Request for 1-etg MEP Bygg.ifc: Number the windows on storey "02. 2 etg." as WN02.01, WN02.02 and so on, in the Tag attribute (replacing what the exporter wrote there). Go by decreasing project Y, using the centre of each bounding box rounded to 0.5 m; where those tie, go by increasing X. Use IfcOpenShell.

First a look at what the model holds.

```python
import ifcopenshell
import ifcopenshell.util.element
import ifcopenshell.util.placement

model = ifcopenshell.open("1-etg MEP Bygg.ifc")
print(model.schema)
storey = next(s for s in model.by_type("IfcBuildingStorey") if s.Name == "02. 2 etg.")
windows = [e for e in ifcopenshell.util.element.get_decomposition(storey) if e.is_a("IfcWindow")]
for e in sorted(windows, key=lambda e: e.id()):
    origin = ifcopenshell.util.placement.get_local_placement(e.ObjectPlacement)[:3, 3]
    print(e.id(), e.Tag, e.Name, origin.round(2) + 0.0, sep=" | ")
```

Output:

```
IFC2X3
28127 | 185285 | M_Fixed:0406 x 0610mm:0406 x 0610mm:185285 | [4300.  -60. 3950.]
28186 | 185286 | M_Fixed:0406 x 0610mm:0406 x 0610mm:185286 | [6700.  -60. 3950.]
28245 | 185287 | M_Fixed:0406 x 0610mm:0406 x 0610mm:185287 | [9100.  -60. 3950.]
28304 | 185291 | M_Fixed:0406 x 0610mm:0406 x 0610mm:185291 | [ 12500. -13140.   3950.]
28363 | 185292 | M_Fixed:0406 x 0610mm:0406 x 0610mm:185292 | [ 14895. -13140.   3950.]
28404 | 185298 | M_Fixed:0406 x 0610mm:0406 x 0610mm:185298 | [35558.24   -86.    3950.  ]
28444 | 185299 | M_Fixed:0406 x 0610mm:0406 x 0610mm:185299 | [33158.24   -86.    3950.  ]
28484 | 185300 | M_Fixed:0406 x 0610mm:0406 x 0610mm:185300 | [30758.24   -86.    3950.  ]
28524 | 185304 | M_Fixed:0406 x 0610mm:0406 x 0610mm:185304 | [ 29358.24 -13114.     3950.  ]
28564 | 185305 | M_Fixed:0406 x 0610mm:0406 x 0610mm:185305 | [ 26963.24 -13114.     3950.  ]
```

```python
import ifcopenshell
import ifcopenshell.geom
import ifcopenshell.util.element
import ifcopenshell.util.shape

model = ifcopenshell.open("1-etg MEP Bygg.ifc")
settings = ifcopenshell.geom.settings()
settings.set("use-world-coords", True)


def centre(element):
    shape = ifcopenshell.geom.create_shape(settings, element)
    return ifcopenshell.util.shape.get_bbox_centroid(shape.geometry)


storey = next(s for s in model.by_type("IfcBuildingStorey") if s.Name == "02. 2 etg.")
windows = [e for e in ifcopenshell.util.element.get_decomposition(storey) if e.is_a("IfcWindow")]

# Insertion points can sit at a corner or the storey origin, so sort by the geometry (in metres).
centres = {e: centre(e) for e in windows}
windows.sort(key=lambda e: (-round(centres[e][1] / 0.5), centres[e][0]))

for i, e in enumerate(windows, start=1):
    number = f"WN02.{i:02d}"
    e.Tag = number
    print(e.id(), number)

model.write("1-etg MEP Bygg_rev.ifc")
```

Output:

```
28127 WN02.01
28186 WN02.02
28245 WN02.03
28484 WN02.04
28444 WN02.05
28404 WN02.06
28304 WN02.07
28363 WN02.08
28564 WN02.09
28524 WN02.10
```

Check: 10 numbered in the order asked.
